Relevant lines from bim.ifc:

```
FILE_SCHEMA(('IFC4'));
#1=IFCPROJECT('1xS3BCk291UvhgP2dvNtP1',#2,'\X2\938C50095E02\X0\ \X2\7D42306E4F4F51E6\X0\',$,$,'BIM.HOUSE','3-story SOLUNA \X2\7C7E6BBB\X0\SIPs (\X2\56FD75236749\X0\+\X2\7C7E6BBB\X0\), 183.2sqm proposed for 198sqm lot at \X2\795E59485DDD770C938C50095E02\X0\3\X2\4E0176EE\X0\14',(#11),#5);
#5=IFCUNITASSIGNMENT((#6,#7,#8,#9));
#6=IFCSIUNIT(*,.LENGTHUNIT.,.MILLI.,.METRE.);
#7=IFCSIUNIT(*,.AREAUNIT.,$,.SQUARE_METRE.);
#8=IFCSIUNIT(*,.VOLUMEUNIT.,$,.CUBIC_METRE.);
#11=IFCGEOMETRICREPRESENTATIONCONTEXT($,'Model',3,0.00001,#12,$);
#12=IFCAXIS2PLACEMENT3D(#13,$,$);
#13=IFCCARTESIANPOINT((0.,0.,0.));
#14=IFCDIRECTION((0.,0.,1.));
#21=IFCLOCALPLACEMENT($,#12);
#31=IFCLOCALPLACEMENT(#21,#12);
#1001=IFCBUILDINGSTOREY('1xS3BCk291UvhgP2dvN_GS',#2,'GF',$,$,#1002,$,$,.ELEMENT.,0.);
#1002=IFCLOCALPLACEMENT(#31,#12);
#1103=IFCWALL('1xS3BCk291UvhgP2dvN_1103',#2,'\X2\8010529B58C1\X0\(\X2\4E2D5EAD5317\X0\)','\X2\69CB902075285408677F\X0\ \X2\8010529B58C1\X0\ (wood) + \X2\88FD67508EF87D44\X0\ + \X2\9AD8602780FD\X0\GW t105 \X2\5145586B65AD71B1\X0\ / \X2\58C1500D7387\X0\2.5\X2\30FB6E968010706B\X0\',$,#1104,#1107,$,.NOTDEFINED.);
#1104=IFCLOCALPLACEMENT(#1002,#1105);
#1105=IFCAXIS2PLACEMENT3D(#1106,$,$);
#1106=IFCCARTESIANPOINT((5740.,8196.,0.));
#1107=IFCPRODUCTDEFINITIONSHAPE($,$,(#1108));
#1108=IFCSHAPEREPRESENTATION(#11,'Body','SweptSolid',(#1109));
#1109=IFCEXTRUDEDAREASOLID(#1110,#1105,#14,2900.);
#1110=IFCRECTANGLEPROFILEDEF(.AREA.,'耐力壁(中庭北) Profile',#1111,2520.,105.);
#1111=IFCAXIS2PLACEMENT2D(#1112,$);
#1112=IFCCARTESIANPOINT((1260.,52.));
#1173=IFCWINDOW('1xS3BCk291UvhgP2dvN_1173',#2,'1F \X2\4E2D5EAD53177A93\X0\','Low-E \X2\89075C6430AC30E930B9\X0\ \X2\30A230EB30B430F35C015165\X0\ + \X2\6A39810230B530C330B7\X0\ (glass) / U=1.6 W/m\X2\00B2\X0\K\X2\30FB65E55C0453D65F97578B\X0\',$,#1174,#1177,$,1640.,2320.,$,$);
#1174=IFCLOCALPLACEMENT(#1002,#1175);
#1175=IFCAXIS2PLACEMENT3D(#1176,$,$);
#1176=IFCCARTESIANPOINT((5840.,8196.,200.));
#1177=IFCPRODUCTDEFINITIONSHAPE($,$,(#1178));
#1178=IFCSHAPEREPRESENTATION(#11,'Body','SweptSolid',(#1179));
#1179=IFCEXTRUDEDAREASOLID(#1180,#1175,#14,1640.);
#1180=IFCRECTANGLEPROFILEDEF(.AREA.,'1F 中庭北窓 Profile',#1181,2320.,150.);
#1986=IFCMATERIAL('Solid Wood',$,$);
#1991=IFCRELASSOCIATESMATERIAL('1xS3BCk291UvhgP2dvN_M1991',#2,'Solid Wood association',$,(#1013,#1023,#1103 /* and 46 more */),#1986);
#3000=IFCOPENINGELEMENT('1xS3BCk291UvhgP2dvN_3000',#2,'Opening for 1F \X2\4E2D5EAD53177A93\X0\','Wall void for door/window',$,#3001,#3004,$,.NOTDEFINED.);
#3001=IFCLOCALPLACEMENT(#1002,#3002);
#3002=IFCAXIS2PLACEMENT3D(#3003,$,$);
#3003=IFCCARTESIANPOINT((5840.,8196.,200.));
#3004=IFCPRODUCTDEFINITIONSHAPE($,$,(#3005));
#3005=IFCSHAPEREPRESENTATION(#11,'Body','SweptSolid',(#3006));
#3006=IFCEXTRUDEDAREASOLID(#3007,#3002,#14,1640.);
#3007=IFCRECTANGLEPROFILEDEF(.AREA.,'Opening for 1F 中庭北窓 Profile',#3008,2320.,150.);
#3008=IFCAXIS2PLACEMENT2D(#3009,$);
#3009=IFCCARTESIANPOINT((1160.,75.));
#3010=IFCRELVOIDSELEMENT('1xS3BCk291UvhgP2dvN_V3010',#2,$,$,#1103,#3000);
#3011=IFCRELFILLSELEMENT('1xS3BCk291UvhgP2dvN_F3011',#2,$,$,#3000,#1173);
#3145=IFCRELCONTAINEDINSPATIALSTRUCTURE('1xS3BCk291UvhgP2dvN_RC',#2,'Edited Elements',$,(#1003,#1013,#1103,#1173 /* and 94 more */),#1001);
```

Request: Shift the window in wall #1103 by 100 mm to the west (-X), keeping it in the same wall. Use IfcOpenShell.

```python
import ifcopenshell
import ifcopenshell.api.geometry
import ifcopenshell.util.placement
import ifcopenshell.util.unit

model = ifcopenshell.open("bim.ifc")
unit_scale = ifcopenshell.util.unit.calculate_unit_scale(model)

window = model.by_guid("1xS3BCk291UvhgP2dvN_1173")
opening = window.FillsVoids[0].RelatingOpeningElement
wall = opening.VoidsElements[0].RelatingBuildingElement

wall_matrix = ifcopenshell.util.placement.get_local_placement(wall.ObjectPlacement)
shift = wall_matrix[:3, 0] * -0.1 / unit_scale
before = ifcopenshell.util.placement.get_local_placement(window.ObjectPlacement)[:3, 3].copy()

# The window is not placed relative to its opening, so move both.
for product in (opening, window):
    matrix = ifcopenshell.util.placement.get_local_placement(product.ObjectPlacement)
    matrix[:3, 3] += shift
    ifcopenshell.api.geometry.edit_object_placement(model, product=product, matrix=matrix, is_si=False)

after = ifcopenshell.util.placement.get_local_placement(window.ObjectPlacement)[:3, 3]
print("window moved by", (after - before).round(3) + 0.0)

model.write("bim-out.ifc")
```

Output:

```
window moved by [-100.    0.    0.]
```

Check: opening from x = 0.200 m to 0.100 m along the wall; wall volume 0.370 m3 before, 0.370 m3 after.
